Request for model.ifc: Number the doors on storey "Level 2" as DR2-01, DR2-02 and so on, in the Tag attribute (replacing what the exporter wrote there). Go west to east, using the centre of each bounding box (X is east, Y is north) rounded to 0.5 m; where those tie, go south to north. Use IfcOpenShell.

First a look at what the model holds.

```python
import ifcopenshell
import ifcopenshell.util.element
import ifcopenshell.util.placement

model = ifcopenshell.open("model.ifc")
print(model.schema)
storey = next(s for s in model.by_type("IfcBuildingStorey") if s.Name == "Level 2")
doors = [e for e in ifcopenshell.util.element.get_decomposition(storey) if e.is_a("IfcDoor")]
for e in sorted(doors, key=lambda e: e.id()):
    origin = ifcopenshell.util.placement.get_local_placement(e.ObjectPlacement)[:3, 3]
    print(e.id(), e.Tag, e.Name, origin.round(2) + 0.0, sep=" | ")
```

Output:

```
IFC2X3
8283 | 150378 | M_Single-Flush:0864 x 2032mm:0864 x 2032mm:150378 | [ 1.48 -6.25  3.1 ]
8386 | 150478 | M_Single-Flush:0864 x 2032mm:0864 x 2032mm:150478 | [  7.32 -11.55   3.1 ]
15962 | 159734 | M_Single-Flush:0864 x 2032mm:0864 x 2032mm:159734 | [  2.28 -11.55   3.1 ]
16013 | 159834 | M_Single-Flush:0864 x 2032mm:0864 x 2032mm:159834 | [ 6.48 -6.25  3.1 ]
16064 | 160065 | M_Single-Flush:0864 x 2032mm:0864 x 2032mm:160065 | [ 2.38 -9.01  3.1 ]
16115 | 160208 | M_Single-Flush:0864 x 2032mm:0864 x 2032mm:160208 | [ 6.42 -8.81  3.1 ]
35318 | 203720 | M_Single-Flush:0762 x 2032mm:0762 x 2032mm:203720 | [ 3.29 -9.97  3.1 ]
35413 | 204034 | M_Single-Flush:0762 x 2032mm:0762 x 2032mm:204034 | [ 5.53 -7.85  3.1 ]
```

```python
import ifcopenshell
import ifcopenshell.geom
import ifcopenshell.util.element
import ifcopenshell.util.shape

model = ifcopenshell.open("model.ifc")
settings = ifcopenshell.geom.settings()
settings.set("use-world-coords", True)


def centre(element):
    shape = ifcopenshell.geom.create_shape(settings, element)
    return ifcopenshell.util.shape.get_bbox_centroid(shape.geometry)


storey = next(s for s in model.by_type("IfcBuildingStorey") if s.Name == "Level 2")
doors = [e for e in ifcopenshell.util.element.get_decomposition(storey) if e.is_a("IfcDoor")]

# Insertion points can sit at a corner or the storey origin, so sort by the geometry (in metres).
centres = {e: centre(e) for e in doors}
doors.sort(key=lambda e: (round(centres[e][0] / 0.5), centres[e][1]))

for i, e in enumerate(doors, start=1):
    number = f"DR2-{i:02d}"
    e.Tag = number
    print(e.id(), number)

model.write("model_edited.ifc")
```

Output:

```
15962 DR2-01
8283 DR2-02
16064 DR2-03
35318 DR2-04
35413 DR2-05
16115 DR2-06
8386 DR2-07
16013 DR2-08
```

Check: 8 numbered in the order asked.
